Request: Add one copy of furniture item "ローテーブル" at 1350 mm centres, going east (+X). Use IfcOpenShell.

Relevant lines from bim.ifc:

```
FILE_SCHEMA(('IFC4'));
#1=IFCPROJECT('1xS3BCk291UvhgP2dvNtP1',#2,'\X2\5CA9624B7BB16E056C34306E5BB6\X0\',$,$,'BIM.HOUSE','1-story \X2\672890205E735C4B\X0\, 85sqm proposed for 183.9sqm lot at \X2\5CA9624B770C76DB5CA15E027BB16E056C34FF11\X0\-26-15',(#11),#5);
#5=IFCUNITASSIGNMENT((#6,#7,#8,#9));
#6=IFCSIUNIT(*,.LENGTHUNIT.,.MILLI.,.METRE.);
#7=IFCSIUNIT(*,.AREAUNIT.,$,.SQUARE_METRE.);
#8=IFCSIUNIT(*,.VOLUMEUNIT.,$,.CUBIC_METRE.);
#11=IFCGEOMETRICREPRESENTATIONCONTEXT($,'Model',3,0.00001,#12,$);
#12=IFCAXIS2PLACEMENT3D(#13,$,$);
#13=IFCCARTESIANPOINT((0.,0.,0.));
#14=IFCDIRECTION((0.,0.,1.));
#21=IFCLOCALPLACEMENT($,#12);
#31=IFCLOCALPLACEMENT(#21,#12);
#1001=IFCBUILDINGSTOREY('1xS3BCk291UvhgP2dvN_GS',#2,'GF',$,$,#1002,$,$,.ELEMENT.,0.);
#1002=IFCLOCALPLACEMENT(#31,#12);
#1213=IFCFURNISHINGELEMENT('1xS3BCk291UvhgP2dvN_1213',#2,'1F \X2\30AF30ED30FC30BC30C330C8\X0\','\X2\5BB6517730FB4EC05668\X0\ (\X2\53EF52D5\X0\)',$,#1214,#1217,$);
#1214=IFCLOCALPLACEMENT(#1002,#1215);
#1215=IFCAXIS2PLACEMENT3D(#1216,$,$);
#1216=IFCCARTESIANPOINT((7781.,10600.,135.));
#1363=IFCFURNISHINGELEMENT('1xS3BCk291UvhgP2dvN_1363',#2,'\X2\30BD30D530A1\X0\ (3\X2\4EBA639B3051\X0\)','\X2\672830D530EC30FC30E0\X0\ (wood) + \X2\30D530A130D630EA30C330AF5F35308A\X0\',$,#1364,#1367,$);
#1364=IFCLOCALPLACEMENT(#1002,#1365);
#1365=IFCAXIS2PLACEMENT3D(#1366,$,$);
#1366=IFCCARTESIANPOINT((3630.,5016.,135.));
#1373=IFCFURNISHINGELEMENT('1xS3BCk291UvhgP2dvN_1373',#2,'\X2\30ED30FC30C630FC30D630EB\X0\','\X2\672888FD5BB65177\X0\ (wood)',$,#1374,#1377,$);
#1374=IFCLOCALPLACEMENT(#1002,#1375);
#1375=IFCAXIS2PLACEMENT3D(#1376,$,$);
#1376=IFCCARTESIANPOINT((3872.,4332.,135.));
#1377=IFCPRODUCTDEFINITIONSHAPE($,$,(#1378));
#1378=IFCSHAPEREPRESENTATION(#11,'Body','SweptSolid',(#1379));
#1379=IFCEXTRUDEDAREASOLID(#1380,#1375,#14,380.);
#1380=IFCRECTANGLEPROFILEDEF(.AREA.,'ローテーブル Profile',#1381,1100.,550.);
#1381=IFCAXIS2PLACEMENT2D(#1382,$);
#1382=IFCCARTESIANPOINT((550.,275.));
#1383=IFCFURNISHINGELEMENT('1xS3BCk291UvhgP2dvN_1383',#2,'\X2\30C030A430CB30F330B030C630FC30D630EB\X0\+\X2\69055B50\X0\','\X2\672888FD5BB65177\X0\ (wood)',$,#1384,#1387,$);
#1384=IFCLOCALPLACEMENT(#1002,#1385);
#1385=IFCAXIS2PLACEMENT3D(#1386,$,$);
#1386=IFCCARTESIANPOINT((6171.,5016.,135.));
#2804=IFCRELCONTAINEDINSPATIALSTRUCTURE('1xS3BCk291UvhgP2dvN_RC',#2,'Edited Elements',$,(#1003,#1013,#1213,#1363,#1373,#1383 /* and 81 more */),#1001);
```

```python
import numpy as np
import ifcopenshell
import ifcopenshell.api.geometry
import ifcopenshell.api.root
import ifcopenshell.util.element
import ifcopenshell.util.placement
import ifcopenshell.util.unit

model = ifcopenshell.open("bim.ifc")
unit_scale = ifcopenshell.util.unit.calculate_unit_scale(model)


def reuse_history(source, copy):
    """copy_class also copies each property set's owner history, people and application; keep the originals."""
    for rel in copy.IsDefinedBy:
        if rel.is_a("IfcRelDefinesByProperties") and (history := rel.RelatingPropertyDefinition.OwnerHistory):
            rel.RelatingPropertyDefinition.OwnerHistory = source.OwnerHistory
            ifcopenshell.util.element.remove_deep2(model, history)


source = model.by_guid("1xS3BCk291UvhgP2dvN_1373")
base = ifcopenshell.util.placement.get_local_placement(source.ObjectPlacement)
step = np.array([1.0, 0.0, 0.0]) * 1.35 / unit_scale

for i in range(1, 2):
    copy = ifcopenshell.api.root.copy_class(model, product=source)
    copy.Representation = ifcopenshell.util.element.copy_deep(
        model, source.Representation, exclude=["IfcGeometricRepresentationContext", "IfcRepresentationMap"]
    )
    reuse_history(source, copy)
    matrix = base.copy()
    matrix[:3, 3] += i * step
    print("added at", matrix[:3, 3].round(3) + 0.0)
    ifcopenshell.api.geometry.edit_object_placement(model, product=copy, matrix=matrix, is_si=False)

model.write("bim-out.ifc")
```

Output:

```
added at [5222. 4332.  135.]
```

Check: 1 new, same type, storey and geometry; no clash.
